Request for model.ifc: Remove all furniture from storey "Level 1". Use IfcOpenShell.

First a look at what the model holds.

```python
import ifcopenshell
import ifcopenshell.util.element

model = ifcopenshell.open("model.ifc")
print(model.schema)
storey = next(s for s in model.by_type("IfcBuildingStorey") if s.Name == "Level 1")
furniture = [e for e in ifcopenshell.util.element.get_decomposition(storey) if e.is_a("IfcFurnishingElement")]
seen = {}
for e in furniture:
    element_type = ifcopenshell.util.element.get_type(e)
    name = element_type.Name if element_type not in (None, e) else None
    seen[name] = seen.get(name, 0) + 1
for name, count in sorted(seen.items(), key=str):
    print(count, "x", name)
```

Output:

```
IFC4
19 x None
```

```python
import ifcopenshell
import ifcopenshell.api.root
import ifcopenshell.util.element

model = ifcopenshell.open("model.ifc")

storey = next(s for s in model.by_type("IfcBuildingStorey") if s.Name == "Level 1")
furniture = [e for e in ifcopenshell.util.element.get_decomposition(storey) if e.is_a("IfcFurnishingElement")]

for e in furniture:
    ifcopenshell.api.root.remove_product(model, product=e)
print(len(furniture), "removed")

model.write("model_edited.ifc")
```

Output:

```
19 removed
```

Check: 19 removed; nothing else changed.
